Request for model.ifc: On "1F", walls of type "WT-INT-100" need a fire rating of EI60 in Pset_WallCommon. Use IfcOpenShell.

First a look at what the model holds.

```python
import ifcopenshell
import ifcopenshell.util.element

model = ifcopenshell.open("model.ifc")
print(model.schema)
storey = next(s for s in model.by_type("IfcBuildingStorey") if s.Name == "1F")
walls = [e for e in ifcopenshell.util.element.get_decomposition(storey) if e.is_a("IfcWall")]
seen = {}
for e in walls:
    element_type = ifcopenshell.util.element.get_type(e)
    key = (element_type.Name if element_type != e and element_type else None, ifcopenshell.util.element.get_pset(e, "Pset_WallCommon", "FireRating"))
    seen[key] = seen.get(key, 0) + 1
for (name, value), count in sorted(seen.items(), key=str):
    print(count, "x", name, "|", value)
```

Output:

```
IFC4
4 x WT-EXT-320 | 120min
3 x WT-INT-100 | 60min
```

```python
import ifcopenshell
import ifcopenshell.api.pset
import ifcopenshell.util.element

model = ifcopenshell.open("model.ifc")

storey = next(s for s in model.by_type("IfcBuildingStorey") if s.Name == "1F")
walls = [e for e in ifcopenshell.util.element.get_decomposition(storey) if e.is_a("IfcWall")]

count = 0
for e in walls:
    element_type = ifcopenshell.util.element.get_type(e)
    if element_type in (None, e) or element_type.Name != "WT-INT-100":
        continue
    # add_pset returns the element's existing set when there is one.
    pset = ifcopenshell.api.pset.add_pset(model, product=e, name="Pset_WallCommon")
    ifcopenshell.api.pset.edit_pset(model, pset=pset, properties={"FireRating": "EI60"})
    count += 1

print(count, "walls updated")

model.write("model_v2.ifc")
```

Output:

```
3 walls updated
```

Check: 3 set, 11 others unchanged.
